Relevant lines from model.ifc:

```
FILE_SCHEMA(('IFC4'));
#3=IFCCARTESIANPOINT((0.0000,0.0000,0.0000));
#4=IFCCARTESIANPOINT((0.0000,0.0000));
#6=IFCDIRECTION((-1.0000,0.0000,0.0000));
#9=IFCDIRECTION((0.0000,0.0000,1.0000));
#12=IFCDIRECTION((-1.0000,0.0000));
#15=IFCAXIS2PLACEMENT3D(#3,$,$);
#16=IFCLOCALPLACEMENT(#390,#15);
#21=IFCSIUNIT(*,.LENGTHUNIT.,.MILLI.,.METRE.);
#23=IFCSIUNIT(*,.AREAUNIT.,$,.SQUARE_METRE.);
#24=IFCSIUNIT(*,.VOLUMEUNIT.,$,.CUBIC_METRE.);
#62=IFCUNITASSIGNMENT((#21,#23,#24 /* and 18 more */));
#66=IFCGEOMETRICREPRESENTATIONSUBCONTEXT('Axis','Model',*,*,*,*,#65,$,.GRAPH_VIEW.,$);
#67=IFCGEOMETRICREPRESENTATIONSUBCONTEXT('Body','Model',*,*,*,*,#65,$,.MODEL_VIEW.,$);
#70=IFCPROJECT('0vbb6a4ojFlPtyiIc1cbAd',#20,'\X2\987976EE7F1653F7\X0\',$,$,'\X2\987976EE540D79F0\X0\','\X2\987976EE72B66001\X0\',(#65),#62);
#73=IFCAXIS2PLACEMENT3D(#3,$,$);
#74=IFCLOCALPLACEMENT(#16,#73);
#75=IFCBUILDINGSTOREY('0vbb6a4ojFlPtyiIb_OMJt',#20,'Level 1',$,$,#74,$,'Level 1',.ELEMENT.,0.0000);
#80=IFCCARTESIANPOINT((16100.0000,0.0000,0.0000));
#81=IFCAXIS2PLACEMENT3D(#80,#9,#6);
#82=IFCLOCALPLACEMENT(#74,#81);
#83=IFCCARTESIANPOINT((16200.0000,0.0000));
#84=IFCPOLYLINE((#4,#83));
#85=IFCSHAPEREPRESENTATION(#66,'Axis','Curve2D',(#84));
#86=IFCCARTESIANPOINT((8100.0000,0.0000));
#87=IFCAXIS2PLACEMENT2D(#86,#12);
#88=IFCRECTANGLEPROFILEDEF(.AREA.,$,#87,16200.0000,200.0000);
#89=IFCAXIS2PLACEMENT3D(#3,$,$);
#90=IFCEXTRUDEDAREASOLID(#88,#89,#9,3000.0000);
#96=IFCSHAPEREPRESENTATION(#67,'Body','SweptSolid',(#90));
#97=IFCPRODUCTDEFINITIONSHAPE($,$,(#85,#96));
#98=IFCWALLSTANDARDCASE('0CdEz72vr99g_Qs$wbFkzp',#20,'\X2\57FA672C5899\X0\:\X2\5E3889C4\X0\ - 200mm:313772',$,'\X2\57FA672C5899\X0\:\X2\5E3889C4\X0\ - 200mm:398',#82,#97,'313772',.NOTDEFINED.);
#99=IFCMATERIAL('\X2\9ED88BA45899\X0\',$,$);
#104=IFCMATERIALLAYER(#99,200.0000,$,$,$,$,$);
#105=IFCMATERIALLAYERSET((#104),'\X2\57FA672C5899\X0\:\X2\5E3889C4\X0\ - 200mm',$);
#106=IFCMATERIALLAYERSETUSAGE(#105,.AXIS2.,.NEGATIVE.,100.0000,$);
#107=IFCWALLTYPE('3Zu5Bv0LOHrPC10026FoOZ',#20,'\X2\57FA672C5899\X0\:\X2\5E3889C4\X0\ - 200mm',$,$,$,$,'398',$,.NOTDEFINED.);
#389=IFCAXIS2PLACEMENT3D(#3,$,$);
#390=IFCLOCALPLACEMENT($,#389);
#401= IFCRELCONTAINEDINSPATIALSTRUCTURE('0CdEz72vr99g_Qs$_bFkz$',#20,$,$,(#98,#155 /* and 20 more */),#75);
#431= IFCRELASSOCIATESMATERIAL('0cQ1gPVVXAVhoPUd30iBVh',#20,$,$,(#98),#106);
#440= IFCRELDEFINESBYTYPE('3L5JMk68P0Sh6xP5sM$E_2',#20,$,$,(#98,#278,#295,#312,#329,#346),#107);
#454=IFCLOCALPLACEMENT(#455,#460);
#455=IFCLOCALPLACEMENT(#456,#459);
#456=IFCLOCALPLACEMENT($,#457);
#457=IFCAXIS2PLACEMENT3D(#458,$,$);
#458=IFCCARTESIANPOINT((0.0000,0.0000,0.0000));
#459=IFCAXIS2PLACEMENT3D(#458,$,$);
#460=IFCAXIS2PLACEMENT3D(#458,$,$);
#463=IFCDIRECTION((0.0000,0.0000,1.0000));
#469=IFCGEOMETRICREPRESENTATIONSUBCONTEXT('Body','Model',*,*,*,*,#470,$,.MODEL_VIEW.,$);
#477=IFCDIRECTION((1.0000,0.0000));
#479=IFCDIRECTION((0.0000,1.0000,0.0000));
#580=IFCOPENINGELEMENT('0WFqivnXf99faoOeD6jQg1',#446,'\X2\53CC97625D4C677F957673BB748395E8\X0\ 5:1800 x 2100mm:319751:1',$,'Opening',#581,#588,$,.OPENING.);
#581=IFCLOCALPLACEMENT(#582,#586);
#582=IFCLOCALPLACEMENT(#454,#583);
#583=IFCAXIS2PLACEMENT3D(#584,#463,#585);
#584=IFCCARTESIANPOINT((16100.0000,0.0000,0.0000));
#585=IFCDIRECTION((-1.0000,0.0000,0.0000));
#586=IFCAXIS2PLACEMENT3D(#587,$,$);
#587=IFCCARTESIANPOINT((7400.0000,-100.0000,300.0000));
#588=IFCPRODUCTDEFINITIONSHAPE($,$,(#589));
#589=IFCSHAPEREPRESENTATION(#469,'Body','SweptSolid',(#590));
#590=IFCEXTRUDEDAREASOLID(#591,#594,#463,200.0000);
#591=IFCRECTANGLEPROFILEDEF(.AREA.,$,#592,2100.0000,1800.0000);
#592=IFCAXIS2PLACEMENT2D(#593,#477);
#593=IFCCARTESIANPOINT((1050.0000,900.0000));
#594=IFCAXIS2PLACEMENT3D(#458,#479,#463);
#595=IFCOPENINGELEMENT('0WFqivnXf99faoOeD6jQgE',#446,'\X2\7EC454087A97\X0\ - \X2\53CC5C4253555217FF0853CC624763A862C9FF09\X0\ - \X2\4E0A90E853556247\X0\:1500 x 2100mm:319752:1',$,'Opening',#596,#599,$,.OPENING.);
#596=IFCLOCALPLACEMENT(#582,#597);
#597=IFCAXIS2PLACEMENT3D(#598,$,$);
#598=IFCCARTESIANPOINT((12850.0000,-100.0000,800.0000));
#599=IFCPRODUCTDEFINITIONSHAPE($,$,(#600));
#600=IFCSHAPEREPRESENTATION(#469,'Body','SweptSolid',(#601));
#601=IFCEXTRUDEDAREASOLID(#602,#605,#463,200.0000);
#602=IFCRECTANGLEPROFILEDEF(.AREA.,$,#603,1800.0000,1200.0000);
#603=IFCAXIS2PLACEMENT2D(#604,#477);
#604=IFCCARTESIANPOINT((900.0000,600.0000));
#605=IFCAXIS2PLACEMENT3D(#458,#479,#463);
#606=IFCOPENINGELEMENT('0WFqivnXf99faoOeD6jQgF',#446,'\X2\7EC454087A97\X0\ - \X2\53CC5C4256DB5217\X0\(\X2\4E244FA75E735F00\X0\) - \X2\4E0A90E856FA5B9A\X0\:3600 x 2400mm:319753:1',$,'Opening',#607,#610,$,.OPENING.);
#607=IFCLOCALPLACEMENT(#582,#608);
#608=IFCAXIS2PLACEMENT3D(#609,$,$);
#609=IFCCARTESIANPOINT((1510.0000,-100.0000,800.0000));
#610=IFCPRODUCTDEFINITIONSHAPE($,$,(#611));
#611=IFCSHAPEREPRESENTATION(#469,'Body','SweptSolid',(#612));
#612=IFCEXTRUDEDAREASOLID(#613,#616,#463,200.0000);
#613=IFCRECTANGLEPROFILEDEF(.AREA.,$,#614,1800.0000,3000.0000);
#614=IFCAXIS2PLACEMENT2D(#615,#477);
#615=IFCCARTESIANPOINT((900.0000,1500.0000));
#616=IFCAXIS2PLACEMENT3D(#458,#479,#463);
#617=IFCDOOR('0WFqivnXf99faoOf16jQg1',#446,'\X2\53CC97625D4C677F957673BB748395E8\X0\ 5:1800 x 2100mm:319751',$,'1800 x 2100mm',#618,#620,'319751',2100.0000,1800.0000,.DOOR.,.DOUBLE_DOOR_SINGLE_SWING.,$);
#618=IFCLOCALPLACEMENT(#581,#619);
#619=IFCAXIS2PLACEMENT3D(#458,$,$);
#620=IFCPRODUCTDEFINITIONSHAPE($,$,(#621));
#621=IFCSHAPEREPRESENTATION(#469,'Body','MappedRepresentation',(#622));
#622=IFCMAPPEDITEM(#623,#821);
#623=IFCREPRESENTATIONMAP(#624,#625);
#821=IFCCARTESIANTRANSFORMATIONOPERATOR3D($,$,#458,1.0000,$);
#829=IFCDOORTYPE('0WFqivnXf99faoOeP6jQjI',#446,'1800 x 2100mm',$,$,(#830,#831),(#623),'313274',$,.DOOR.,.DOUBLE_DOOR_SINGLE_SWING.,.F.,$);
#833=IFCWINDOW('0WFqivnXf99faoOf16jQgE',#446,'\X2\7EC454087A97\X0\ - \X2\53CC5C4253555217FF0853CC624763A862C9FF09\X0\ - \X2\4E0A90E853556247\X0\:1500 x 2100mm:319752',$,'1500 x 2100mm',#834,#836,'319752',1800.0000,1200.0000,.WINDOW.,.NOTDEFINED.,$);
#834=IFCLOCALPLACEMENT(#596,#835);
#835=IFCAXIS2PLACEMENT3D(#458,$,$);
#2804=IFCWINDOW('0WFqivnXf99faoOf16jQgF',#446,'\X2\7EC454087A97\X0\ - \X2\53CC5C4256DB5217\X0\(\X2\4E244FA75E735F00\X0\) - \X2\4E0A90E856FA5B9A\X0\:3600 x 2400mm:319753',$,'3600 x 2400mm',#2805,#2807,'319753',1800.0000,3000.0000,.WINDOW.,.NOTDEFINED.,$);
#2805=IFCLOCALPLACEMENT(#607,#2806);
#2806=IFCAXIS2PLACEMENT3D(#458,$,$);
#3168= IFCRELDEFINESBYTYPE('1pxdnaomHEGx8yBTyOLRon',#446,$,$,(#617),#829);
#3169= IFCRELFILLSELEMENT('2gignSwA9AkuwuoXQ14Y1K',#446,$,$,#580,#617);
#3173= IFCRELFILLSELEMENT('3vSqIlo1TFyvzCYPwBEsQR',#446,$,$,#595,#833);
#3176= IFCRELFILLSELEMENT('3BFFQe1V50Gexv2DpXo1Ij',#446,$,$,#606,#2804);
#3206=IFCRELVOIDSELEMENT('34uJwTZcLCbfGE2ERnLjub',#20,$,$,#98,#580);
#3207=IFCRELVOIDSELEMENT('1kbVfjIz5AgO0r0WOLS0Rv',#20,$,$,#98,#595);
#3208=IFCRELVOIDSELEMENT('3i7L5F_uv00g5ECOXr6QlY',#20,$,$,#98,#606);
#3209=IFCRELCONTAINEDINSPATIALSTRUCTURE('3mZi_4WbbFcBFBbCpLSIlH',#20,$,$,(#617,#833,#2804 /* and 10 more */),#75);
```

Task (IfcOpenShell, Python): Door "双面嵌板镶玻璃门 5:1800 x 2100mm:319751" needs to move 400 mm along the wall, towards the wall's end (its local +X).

```python
import ifcopenshell
import ifcopenshell.api.geometry
import ifcopenshell.util.placement
import ifcopenshell.util.unit

model = ifcopenshell.open("model.ifc")
unit_scale = ifcopenshell.util.unit.calculate_unit_scale(model)

door = model.by_guid("0WFqivnXf99faoOf16jQg1")
opening = door.FillsVoids[0].RelatingOpeningElement
wall = opening.VoidsElements[0].RelatingBuildingElement

wall_matrix = ifcopenshell.util.placement.get_local_placement(wall.ObjectPlacement)
shift = wall_matrix[:3, 0] * 0.4 / unit_scale
before = ifcopenshell.util.placement.get_local_placement(door.ObjectPlacement)[:3, 3].copy()

# The door is placed relative to its opening, so it follows when the opening moves.
matrix = ifcopenshell.util.placement.get_local_placement(opening.ObjectPlacement)
matrix[:3, 3] += shift
ifcopenshell.api.geometry.edit_object_placement(
    model, product=opening, matrix=matrix, is_si=False, should_transform_children=True
)

after = ifcopenshell.util.placement.get_local_placement(door.ObjectPlacement)[:3, 3]
print("door moved by", (after - before).round(3) + 0.0)

model.write("model_rev.ifc")
```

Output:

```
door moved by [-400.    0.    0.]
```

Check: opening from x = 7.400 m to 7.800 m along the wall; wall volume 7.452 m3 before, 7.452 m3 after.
